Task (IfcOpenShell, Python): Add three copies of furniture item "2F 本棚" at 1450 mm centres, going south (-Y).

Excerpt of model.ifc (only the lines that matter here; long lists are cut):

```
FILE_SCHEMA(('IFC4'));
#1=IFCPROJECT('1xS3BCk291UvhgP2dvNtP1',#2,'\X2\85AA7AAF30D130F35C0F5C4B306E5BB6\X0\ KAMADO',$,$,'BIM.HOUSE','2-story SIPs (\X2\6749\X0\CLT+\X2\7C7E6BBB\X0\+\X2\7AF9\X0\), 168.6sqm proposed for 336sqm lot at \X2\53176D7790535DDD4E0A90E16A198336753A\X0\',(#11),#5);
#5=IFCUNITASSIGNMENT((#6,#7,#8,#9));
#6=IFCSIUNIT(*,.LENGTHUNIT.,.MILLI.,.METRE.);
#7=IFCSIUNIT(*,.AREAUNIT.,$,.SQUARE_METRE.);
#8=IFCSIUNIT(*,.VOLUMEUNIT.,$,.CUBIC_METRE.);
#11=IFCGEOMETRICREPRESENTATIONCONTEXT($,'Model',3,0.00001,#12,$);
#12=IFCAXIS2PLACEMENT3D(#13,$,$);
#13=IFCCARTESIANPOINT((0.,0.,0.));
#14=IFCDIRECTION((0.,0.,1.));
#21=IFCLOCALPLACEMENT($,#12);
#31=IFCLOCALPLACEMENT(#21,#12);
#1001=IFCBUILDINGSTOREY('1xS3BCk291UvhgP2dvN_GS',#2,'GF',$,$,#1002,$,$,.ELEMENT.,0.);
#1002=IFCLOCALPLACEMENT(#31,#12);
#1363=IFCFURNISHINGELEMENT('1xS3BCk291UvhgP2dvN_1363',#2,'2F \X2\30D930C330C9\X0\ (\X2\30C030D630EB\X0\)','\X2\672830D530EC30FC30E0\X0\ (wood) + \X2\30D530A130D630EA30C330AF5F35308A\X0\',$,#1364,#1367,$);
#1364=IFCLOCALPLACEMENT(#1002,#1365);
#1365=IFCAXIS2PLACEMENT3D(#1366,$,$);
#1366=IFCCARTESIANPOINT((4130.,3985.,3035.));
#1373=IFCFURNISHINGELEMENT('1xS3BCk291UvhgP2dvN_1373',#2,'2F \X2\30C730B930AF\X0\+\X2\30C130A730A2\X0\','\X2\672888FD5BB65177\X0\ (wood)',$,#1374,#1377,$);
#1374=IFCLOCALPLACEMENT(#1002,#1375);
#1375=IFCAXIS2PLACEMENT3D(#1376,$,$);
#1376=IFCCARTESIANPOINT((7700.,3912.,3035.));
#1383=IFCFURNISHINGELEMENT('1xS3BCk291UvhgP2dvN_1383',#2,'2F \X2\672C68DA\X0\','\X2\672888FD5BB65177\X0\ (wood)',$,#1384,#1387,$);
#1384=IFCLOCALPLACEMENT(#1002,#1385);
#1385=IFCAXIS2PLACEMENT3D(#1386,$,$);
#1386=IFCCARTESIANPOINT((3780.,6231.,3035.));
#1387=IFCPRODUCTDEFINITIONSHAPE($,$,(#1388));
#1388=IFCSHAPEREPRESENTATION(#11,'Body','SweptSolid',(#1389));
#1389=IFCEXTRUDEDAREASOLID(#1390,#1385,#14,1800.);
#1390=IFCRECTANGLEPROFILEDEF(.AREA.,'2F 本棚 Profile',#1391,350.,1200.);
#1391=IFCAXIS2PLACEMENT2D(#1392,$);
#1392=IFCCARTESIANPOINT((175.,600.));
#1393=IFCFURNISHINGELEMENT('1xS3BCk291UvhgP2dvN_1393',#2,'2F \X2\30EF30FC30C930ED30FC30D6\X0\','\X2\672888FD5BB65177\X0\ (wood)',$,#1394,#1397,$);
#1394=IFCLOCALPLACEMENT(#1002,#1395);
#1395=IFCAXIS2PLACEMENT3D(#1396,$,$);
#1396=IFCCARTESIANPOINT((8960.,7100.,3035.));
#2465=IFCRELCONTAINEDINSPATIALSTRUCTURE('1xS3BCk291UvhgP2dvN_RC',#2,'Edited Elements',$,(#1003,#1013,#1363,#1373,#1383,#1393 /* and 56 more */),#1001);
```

```python
import numpy as np
import ifcopenshell
import ifcopenshell.api.geometry
import ifcopenshell.api.root
import ifcopenshell.util.element
import ifcopenshell.util.placement

model = ifcopenshell.open("model.ifc")


def reuse_history(source, copy):
    """copy_class also copies each property set's owner history, people and application; keep the originals."""
    for rel in copy.IsDefinedBy:
        if rel.is_a("IfcRelDefinesByProperties") and (history := rel.RelatingPropertyDefinition.OwnerHistory):
            rel.RelatingPropertyDefinition.OwnerHistory = source.OwnerHistory
            ifcopenshell.util.element.remove_deep2(model, history)


source = model.by_guid("1xS3BCk291UvhgP2dvN_1383")
base = ifcopenshell.util.placement.get_local_placement(source.ObjectPlacement)
step = np.array([0.0, -1.0, 0.0]) * 1450.0

for i in range(1, 4):
    copy = ifcopenshell.api.root.copy_class(model, product=source)
    copy.Representation = ifcopenshell.util.element.copy_deep(
        model, source.Representation, exclude=["IfcGeometricRepresentationContext", "IfcRepresentationMap"]
    )
    reuse_history(source, copy)
    matrix = base.copy()
    matrix[:3, 3] += i * step
    print("added at", matrix[:3, 3].round(3) + 0.0)
    ifcopenshell.api.geometry.edit_object_placement(model, product=copy, matrix=matrix, is_si=False)

model.write("model_rev.ifc")
```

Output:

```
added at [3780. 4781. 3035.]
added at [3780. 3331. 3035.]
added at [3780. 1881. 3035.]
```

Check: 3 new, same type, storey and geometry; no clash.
